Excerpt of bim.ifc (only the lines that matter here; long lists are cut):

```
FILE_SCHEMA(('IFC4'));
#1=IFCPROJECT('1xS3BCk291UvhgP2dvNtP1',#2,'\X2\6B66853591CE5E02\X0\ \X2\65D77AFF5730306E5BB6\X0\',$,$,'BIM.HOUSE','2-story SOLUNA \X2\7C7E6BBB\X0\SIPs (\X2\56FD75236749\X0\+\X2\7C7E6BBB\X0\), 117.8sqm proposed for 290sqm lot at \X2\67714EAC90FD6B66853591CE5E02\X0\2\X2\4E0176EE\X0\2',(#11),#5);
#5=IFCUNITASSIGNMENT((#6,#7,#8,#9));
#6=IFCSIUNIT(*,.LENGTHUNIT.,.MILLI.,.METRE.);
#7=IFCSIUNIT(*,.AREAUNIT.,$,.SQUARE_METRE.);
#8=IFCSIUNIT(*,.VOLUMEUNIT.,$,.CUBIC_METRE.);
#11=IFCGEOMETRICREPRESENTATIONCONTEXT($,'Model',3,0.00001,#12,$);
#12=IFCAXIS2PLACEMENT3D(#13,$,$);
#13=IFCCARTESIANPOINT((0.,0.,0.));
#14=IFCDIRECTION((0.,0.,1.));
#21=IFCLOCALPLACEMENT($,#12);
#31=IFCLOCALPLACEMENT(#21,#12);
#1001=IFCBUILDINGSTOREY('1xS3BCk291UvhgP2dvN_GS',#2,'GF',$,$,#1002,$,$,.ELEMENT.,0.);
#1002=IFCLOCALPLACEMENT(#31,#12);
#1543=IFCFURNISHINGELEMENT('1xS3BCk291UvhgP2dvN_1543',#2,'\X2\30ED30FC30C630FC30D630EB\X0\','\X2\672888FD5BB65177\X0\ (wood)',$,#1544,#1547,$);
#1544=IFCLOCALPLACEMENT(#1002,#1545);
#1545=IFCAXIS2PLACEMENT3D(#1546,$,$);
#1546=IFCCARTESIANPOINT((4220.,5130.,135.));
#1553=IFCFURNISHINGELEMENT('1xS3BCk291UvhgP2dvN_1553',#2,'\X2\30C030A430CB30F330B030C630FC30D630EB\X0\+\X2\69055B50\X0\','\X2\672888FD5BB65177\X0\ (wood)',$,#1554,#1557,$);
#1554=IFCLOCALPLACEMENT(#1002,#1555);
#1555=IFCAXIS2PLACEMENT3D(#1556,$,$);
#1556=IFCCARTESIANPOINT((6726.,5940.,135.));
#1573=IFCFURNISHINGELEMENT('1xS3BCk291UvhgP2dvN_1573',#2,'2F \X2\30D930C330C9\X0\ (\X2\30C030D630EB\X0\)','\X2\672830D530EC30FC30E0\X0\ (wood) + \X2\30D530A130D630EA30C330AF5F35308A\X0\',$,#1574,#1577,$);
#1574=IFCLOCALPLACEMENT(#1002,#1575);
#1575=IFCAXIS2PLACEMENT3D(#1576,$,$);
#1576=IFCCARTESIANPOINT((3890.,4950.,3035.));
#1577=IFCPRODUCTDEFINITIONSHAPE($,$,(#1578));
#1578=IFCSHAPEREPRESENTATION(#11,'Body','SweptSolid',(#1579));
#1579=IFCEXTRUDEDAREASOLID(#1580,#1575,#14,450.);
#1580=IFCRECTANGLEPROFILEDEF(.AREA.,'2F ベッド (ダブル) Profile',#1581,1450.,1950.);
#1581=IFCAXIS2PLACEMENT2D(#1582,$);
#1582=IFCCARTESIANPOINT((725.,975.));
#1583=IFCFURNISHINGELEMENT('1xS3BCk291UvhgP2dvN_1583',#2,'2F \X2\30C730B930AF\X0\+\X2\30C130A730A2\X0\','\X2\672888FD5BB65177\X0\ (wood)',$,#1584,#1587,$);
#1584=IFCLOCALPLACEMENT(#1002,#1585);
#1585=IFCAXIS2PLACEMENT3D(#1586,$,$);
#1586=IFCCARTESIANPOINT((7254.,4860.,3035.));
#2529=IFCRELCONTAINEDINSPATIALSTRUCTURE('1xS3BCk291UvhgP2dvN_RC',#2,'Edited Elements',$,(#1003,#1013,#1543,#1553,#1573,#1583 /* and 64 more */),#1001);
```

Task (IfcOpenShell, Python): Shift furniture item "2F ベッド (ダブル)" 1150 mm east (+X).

```python
import ifcopenshell
import ifcopenshell.api.geometry
import ifcopenshell.util.placement

model = ifcopenshell.open("bim.ifc")

item = model.by_guid("1xS3BCk291UvhgP2dvN_1573")
matrix = ifcopenshell.util.placement.get_local_placement(item.ObjectPlacement)
matrix[0, 3] += 1150.0
ifcopenshell.api.geometry.edit_object_placement(model, product=item, matrix=matrix, is_si=False)

print(ifcopenshell.util.placement.get_local_placement(item.ObjectPlacement).round(3) + 0.0)

model.write("bim_v2.ifc")
```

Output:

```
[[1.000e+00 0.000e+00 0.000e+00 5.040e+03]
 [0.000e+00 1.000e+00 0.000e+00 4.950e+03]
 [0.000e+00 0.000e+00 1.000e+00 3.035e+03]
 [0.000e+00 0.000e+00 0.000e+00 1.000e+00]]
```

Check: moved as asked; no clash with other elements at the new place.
